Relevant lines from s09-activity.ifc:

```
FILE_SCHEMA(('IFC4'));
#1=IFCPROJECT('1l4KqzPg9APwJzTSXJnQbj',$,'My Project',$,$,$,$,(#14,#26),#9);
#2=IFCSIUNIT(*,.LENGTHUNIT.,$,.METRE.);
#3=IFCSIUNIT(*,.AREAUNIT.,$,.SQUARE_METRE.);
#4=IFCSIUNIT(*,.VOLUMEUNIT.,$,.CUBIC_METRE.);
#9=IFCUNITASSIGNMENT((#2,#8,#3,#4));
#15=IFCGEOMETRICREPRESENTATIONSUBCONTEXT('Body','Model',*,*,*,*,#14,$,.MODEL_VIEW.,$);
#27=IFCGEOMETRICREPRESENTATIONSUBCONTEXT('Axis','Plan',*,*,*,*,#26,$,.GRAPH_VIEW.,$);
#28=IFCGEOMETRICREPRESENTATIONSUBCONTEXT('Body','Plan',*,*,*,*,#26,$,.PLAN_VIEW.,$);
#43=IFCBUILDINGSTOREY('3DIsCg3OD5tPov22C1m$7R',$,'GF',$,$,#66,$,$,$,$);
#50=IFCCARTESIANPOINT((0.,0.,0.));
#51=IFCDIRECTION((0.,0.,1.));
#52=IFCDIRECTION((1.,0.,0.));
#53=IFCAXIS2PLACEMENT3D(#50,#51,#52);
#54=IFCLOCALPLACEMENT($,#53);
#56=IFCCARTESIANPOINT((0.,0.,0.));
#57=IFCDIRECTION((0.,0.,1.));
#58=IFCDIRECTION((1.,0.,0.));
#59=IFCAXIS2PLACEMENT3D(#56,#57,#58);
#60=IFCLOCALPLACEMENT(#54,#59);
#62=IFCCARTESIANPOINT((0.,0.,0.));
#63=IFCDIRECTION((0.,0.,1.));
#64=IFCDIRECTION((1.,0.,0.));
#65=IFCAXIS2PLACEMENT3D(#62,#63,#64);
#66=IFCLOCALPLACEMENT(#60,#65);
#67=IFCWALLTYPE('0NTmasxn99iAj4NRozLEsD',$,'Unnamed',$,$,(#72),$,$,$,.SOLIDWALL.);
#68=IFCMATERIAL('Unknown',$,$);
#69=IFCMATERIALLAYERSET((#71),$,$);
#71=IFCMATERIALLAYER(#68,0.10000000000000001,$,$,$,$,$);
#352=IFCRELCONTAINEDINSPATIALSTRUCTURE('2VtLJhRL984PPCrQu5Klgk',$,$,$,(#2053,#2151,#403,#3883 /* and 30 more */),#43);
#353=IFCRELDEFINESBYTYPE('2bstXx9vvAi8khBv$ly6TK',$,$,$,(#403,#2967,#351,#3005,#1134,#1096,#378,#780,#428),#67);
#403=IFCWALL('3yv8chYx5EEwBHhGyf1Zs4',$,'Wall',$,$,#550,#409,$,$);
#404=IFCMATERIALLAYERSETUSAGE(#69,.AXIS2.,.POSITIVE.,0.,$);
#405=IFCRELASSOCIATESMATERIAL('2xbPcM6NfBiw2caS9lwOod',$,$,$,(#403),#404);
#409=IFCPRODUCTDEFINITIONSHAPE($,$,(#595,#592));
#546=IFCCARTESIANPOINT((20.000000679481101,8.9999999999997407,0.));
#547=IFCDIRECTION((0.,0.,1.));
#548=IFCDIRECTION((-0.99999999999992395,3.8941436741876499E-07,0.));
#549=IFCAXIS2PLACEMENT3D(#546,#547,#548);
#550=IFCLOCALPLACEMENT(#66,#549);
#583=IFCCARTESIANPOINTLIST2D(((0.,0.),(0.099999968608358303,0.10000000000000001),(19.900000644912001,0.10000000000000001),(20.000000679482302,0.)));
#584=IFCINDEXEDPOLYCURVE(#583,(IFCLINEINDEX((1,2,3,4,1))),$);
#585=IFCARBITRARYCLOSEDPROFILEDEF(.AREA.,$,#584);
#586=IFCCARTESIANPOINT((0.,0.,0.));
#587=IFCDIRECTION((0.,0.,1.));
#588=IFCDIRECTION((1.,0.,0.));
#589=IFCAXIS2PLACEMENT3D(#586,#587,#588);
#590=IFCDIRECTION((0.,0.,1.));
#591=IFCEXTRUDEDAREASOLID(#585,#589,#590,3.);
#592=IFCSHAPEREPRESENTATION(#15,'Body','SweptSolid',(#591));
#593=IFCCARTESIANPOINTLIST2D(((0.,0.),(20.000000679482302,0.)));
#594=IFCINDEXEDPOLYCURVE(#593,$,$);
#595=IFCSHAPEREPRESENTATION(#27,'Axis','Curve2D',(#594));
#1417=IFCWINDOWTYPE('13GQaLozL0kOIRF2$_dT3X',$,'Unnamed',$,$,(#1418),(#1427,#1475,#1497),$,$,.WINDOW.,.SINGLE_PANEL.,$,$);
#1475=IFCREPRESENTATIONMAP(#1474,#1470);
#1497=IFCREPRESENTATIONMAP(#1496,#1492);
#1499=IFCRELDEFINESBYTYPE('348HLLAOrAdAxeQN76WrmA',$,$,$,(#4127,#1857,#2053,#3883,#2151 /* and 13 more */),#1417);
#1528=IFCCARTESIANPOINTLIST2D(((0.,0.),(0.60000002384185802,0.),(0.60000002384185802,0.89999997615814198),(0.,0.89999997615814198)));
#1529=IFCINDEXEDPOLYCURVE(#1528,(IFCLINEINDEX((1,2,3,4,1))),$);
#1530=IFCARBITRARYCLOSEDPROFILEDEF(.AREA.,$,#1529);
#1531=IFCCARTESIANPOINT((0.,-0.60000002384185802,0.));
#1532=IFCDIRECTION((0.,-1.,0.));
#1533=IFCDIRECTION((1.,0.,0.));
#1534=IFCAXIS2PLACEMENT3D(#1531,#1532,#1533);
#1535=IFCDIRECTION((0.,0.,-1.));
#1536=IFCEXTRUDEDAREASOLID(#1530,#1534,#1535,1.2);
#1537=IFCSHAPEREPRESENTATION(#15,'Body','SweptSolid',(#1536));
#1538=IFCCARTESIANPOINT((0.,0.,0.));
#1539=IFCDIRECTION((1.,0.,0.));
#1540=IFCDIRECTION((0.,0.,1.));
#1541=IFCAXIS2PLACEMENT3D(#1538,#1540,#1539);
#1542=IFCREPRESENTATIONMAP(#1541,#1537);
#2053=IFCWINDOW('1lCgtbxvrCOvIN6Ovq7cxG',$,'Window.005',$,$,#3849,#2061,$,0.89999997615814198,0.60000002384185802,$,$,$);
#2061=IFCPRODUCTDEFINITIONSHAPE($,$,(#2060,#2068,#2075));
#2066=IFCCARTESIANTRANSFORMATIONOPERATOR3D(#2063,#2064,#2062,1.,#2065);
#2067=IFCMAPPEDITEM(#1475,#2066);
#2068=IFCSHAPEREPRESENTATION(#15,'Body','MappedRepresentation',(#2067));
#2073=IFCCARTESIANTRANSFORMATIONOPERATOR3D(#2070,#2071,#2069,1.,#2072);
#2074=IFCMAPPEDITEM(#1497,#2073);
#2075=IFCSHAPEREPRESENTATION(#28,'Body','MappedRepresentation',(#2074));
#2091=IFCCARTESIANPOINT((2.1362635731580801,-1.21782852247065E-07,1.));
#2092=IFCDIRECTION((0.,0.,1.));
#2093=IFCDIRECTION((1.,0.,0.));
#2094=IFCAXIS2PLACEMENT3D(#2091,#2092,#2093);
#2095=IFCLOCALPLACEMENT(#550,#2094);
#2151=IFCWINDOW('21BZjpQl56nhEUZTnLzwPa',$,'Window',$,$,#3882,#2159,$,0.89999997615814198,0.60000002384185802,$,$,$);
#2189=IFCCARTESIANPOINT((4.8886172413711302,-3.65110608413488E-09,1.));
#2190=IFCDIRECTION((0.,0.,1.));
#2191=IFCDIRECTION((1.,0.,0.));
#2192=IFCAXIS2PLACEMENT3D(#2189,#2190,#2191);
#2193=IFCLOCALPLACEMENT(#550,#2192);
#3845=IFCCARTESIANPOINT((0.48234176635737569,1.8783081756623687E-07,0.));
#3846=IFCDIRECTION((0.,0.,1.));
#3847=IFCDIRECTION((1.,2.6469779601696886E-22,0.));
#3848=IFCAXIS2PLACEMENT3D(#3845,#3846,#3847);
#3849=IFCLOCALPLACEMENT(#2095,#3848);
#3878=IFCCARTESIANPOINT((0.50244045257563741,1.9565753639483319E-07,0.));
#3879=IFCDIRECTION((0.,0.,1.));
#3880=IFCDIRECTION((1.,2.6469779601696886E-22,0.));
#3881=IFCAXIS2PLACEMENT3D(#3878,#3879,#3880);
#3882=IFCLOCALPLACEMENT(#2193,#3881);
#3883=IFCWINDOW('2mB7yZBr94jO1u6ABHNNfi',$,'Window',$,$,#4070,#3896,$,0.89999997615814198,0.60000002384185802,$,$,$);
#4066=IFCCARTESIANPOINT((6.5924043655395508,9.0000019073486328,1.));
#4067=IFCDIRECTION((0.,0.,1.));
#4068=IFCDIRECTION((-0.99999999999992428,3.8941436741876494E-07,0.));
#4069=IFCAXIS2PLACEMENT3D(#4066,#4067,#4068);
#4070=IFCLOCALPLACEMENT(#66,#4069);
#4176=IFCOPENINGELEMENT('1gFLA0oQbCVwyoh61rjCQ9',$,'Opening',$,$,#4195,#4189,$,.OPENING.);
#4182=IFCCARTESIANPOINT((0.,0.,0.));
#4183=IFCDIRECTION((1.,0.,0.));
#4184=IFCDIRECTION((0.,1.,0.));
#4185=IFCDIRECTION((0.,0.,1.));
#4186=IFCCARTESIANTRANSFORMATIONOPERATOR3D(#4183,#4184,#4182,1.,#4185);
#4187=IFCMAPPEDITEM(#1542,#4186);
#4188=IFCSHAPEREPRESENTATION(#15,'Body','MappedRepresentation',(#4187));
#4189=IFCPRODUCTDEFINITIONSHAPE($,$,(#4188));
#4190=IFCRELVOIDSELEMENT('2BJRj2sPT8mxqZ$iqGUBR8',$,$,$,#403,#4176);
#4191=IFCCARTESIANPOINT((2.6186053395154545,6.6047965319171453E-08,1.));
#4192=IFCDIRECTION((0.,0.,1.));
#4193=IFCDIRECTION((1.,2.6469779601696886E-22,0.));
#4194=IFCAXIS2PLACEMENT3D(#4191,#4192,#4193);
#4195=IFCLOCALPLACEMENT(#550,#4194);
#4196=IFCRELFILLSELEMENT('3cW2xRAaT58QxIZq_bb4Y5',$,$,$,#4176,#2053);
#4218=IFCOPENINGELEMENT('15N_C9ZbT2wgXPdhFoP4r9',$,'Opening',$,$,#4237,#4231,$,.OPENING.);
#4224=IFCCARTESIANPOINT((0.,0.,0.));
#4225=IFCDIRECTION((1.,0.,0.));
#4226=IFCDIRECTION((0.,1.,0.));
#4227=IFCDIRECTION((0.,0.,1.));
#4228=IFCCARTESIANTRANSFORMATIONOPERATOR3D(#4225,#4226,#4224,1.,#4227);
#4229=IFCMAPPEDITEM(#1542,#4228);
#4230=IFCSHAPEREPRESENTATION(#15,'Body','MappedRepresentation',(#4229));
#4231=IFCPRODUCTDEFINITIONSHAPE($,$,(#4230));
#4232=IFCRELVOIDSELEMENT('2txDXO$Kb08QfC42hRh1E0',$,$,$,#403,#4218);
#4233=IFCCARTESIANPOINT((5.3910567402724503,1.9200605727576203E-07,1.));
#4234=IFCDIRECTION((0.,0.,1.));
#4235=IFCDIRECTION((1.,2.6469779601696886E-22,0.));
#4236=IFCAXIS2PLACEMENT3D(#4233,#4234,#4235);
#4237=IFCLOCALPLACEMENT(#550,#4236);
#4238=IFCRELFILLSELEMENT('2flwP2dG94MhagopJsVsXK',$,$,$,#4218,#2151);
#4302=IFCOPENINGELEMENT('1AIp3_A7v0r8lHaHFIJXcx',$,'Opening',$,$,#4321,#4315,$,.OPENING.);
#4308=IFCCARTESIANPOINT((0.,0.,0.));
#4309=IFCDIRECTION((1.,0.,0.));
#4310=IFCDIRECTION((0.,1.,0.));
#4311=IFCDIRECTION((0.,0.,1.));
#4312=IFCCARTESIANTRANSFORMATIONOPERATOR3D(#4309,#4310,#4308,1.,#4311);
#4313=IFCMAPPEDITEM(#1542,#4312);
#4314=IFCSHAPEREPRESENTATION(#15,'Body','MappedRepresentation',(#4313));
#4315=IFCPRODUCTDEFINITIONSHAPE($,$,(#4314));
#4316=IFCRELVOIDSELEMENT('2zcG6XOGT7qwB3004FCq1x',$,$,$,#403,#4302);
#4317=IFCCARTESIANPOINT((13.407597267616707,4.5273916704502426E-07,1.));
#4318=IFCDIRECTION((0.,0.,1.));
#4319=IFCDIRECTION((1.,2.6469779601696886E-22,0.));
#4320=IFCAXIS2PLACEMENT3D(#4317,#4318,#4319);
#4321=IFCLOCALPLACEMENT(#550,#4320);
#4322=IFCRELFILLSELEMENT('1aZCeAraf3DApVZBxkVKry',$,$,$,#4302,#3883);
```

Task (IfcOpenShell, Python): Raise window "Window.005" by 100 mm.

```python
import numpy as np
import ifcopenshell
import ifcopenshell.api.geometry
import ifcopenshell.util.placement
import ifcopenshell.util.unit

model = ifcopenshell.open("s09-activity.ifc")
unit_scale = ifcopenshell.util.unit.calculate_unit_scale(model)

window = model.by_guid("1lCgtbxvrCOvIN6Ovq7cxG")
opening = window.FillsVoids[0].RelatingOpeningElement
dz = 0.1 / unit_scale

shift = np.array([0.0, 0.0, dz])
# The window is not placed relative to its opening, so move both.
for product in (opening, window):
    matrix = ifcopenshell.util.placement.get_local_placement(product.ObjectPlacement)
    matrix[:3, 3] += shift
    ifcopenshell.api.geometry.edit_object_placement(model, product=product, matrix=matrix, is_si=False)

print(f"moved by {dz * unit_scale:+.3f} m")

model.write("s09-activity-out.ifc")
```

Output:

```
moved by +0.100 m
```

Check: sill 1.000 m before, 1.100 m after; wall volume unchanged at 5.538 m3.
